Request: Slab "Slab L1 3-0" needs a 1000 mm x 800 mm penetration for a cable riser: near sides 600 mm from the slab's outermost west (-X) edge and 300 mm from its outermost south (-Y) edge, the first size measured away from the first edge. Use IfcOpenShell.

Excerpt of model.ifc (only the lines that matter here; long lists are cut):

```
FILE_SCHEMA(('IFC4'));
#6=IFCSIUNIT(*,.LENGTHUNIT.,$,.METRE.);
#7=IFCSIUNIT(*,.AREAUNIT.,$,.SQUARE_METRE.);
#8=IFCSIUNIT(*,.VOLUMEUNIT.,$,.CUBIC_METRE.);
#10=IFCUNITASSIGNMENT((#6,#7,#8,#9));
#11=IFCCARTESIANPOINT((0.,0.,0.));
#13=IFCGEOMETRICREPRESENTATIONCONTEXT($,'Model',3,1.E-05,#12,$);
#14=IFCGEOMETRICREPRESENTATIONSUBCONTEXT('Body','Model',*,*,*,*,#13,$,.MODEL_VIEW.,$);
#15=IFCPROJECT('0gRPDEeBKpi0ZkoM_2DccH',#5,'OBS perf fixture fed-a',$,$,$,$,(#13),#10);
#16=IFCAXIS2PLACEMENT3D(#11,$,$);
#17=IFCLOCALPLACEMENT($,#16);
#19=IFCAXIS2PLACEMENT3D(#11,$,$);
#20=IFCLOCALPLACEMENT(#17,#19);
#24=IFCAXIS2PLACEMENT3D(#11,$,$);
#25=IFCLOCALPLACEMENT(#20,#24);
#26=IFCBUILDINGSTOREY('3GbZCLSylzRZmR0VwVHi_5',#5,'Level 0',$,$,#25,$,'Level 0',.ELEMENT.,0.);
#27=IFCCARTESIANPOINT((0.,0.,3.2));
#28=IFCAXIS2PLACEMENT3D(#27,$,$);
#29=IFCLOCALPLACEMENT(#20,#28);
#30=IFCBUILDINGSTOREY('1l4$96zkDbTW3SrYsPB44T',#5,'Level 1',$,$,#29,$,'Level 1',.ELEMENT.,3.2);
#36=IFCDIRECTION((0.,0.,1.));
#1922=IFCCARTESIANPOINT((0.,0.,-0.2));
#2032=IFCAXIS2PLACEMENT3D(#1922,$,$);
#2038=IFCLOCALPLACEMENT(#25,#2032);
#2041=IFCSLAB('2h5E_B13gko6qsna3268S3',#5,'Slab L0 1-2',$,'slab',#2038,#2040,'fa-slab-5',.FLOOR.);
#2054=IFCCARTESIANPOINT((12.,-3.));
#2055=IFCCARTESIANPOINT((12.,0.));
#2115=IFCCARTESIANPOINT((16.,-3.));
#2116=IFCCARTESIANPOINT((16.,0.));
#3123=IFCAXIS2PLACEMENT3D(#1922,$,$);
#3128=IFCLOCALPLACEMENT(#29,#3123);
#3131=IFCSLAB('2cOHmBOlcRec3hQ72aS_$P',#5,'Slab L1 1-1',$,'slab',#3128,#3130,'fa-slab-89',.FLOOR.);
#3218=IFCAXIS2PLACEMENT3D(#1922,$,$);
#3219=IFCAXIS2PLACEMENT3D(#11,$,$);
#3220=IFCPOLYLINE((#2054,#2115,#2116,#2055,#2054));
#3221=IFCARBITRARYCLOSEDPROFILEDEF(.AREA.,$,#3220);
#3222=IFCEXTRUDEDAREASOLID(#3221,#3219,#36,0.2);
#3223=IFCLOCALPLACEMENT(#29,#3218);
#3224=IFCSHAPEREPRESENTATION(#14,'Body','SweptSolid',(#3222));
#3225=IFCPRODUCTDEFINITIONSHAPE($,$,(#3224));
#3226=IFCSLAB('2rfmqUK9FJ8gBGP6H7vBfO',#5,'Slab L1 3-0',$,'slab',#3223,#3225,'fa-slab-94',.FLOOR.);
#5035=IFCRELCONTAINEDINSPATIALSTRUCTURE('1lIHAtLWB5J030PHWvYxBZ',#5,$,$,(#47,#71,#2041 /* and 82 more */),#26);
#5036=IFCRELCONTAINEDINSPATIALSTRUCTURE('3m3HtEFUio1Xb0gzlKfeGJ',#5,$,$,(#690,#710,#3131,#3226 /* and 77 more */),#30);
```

```python
import numpy as np
import ifcopenshell
import ifcopenshell.api.feature
import ifcopenshell.api.geometry
import ifcopenshell.api.root
import ifcopenshell.geom
import ifcopenshell.util.placement
import ifcopenshell.util.representation
import ifcopenshell.util.shape
import ifcopenshell.util.unit

model = ifcopenshell.open("model.ifc")
unit_scale = ifcopenshell.util.unit.calculate_unit_scale(model)
settings = ifcopenshell.geom.settings()


def volume(element):
    """Net volume in cubic metres, openings subtracted."""
    shape = ifcopenshell.geom.create_shape(settings, element)
    return ifcopenshell.util.shape.get_volume(shape.geometry)


slab = model.by_id(3226)
before = volume(slab)

# Extent in the slab's own axes, in metres. The edges named are its -X and -Y sides.
slab_shape = ifcopenshell.geom.create_shape(settings, slab)
vertices = ifcopenshell.util.shape.get_vertices(slab_shape.geometry)
x_min, y_min, bottom = vertices.min(axis=0)
top = vertices[:, 2].max()

opening = ifcopenshell.api.root.create_entity(model, ifc_class="IfcOpeningElement", name="Cable riser opening", predefined_type="OPENING")
context = ifcopenshell.util.representation.get_context(model, "Model", "Body", "MODEL_VIEW")
width, depth = 1, 0.8
outline = [(0.0, 0.0), (width, 0.0), (width, depth), (0.0, depth), (0.0, 0.0)]
# Overshoot both faces by 50 mm so the cut is clean.
shape = ifcopenshell.api.geometry.add_slab_representation(
    model, context=context, depth=top - bottom + 0.1, polyline=outline
)
ifcopenshell.api.geometry.assign_representation(model, product=opening, representation=shape)

matrix = ifcopenshell.util.placement.get_local_placement(slab.ObjectPlacement)
matrix[:, 3] = matrix @ np.append(np.array([x_min + 0.6, y_min + 0.3, bottom - 0.05]) / unit_scale, 1.0)
ifcopenshell.api.geometry.edit_object_placement(model, product=opening, matrix=matrix, is_si=False)
ifcopenshell.api.feature.add_feature(model, feature=opening, element=slab)

after = volume(slab)

print(f"slab volume {before:.3f} -> {after:.3f} m3")

model.write("model_rev.ifc")
```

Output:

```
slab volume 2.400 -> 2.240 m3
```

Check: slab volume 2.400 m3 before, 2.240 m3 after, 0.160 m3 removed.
